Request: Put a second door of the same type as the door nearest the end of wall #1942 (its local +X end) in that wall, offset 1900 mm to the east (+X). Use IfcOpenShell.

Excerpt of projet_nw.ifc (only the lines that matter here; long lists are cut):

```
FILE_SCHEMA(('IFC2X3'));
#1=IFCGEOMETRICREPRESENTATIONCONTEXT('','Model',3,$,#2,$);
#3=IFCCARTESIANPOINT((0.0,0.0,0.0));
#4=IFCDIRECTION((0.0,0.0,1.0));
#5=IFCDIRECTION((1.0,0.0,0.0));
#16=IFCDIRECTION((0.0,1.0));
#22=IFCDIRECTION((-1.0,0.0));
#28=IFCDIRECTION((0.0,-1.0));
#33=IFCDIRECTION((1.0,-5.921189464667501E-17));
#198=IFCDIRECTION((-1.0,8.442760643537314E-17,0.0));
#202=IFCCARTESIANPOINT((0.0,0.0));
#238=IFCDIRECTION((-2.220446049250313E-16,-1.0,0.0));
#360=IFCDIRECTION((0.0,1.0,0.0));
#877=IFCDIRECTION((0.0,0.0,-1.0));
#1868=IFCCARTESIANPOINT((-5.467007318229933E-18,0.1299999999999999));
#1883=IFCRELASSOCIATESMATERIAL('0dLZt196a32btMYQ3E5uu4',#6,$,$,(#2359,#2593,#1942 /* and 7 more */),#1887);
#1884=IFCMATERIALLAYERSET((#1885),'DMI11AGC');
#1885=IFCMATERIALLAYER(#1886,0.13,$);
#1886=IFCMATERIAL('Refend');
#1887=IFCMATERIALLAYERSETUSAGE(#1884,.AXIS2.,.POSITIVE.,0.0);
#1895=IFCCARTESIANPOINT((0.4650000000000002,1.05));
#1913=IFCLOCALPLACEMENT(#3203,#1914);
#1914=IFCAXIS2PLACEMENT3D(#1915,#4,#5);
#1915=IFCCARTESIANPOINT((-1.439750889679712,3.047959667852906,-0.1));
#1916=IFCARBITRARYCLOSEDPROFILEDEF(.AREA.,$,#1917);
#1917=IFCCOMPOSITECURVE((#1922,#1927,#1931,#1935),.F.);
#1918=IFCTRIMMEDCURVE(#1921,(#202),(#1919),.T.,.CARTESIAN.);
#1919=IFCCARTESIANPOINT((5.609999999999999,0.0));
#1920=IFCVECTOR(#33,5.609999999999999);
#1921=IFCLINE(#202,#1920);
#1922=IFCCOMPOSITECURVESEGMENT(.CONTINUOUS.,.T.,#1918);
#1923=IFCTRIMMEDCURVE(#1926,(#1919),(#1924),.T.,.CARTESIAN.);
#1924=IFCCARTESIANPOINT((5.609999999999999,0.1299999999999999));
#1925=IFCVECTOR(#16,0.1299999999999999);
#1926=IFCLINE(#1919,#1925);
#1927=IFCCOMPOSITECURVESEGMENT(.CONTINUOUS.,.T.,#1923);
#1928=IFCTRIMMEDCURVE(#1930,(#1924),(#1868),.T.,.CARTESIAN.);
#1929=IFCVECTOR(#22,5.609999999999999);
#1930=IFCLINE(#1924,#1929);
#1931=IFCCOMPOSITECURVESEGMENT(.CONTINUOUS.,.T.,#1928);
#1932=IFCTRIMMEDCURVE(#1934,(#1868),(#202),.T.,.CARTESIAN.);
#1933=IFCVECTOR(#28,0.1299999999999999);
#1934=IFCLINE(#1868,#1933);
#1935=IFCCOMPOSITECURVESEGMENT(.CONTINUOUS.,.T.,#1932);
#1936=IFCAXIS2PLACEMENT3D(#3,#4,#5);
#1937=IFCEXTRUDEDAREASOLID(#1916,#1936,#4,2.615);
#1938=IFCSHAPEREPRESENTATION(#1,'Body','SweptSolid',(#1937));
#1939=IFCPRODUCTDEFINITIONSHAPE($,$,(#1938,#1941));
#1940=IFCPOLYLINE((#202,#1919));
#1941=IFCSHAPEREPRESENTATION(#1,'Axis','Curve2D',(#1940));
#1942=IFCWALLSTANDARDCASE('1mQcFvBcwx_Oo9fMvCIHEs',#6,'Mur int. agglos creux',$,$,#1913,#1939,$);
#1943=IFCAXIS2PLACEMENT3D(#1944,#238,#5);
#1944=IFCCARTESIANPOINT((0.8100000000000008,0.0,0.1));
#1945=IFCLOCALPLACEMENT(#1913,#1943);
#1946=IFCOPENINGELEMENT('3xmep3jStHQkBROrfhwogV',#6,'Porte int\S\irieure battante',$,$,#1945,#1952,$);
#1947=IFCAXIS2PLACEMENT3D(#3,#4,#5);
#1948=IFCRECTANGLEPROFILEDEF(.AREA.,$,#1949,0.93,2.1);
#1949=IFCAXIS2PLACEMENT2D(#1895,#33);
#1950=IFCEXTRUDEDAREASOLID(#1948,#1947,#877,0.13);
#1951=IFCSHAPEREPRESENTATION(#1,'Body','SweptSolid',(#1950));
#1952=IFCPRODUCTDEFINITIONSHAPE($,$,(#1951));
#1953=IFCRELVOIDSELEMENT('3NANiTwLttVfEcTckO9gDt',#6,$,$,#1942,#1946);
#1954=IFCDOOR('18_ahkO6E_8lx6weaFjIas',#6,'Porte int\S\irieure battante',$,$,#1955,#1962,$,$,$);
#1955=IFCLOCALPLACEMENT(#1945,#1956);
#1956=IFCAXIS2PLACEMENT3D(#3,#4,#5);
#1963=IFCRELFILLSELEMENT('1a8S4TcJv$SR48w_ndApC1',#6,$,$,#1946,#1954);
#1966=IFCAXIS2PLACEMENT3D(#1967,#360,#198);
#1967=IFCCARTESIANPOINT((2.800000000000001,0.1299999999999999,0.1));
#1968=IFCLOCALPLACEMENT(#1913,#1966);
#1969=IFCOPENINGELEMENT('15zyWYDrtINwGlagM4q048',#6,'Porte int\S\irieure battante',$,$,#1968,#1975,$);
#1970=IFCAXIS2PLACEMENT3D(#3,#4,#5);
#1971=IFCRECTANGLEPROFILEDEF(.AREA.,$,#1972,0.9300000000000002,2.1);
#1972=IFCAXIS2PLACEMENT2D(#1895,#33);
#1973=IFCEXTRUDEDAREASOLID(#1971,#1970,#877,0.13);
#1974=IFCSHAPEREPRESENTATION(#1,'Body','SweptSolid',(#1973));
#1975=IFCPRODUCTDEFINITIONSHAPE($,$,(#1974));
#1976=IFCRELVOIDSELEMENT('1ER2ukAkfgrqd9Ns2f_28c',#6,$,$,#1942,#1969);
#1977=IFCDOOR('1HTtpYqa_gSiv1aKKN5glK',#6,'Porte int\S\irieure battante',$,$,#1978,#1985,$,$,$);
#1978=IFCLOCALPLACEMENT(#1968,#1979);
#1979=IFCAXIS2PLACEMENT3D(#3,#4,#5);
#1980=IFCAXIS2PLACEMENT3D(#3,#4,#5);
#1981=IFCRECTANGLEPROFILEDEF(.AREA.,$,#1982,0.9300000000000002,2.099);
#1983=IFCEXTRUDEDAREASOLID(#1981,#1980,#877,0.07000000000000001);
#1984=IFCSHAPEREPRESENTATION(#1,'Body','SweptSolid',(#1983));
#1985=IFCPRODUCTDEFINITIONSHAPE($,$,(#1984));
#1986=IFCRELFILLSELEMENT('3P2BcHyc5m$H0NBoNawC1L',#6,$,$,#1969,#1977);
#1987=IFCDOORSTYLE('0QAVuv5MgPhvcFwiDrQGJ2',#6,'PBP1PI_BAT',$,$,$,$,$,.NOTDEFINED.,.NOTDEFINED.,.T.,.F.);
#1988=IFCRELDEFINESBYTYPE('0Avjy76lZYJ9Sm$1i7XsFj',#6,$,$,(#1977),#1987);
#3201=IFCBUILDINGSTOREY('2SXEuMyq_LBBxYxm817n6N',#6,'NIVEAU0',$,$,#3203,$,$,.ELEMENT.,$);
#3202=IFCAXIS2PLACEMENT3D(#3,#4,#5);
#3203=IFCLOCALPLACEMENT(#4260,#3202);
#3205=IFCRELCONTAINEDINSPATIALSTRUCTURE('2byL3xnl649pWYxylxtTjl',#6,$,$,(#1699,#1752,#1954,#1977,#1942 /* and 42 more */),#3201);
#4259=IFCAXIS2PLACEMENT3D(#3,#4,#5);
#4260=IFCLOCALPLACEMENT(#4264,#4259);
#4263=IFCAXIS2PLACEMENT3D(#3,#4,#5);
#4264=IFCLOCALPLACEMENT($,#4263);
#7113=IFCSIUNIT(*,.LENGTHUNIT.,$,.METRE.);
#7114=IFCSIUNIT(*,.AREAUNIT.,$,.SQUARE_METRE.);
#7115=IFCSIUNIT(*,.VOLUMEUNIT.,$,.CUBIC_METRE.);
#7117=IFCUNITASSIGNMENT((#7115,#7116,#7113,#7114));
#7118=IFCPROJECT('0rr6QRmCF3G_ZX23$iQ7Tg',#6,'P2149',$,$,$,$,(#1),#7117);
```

```python
import ifcopenshell
import ifcopenshell.api.feature
import ifcopenshell.api.geometry
import ifcopenshell.api.root
import ifcopenshell.geom
import ifcopenshell.util.element
import ifcopenshell.util.placement
import ifcopenshell.util.shape
import ifcopenshell.util.unit

model = ifcopenshell.open("projet_nw.ifc")
unit_scale = ifcopenshell.util.unit.calculate_unit_scale(model)
settings = ifcopenshell.geom.settings()


def volume(element):
    """Net volume in cubic metres, openings subtracted."""
    shape = ifcopenshell.geom.create_shape(settings, element)
    return ifcopenshell.util.shape.get_volume(shape.geometry)


door = model.by_guid("1HTtpYqa_gSiv1aKKN5glK")
opening = door.FillsVoids[0].RelatingOpeningElement
wall = opening.VoidsElements[0].RelatingBuildingElement
before = volume(wall)
shift = ifcopenshell.util.placement.get_local_placement(wall.ObjectPlacement)[:3, 0] * 1.9 / unit_scale

# copy_class copies the void relationship, type, container and properties, but no geometry.
new_opening = ifcopenshell.api.root.copy_class(model, product=opening)
new_opening.Representation = ifcopenshell.util.element.copy_deep(
    model, opening.Representation, exclude=["IfcGeometricRepresentationContext", "IfcRepresentationMap"]
)
new_door = ifcopenshell.api.root.copy_class(model, product=door)
new_door.Representation = ifcopenshell.util.element.copy_deep(
    model, door.Representation, exclude=["IfcGeometricRepresentationContext", "IfcRepresentationMap"]
)
fills = ifcopenshell.api.feature.add_filling(model, opening=new_opening, element=new_door)
fills.OwnerHistory = new_door.OwnerHistory  # required in IFC2X3

for old, new in ((opening, new_opening), (door, new_door)):
    matrix = ifcopenshell.util.placement.get_local_placement(old.ObjectPlacement)
    matrix[:3, 3] += shift
    ifcopenshell.api.geometry.edit_object_placement(model, product=new, matrix=matrix, is_si=False)

after = volume(wall)

print(f"wall volume {before:.3f} -> {after:.3f} m3")

model.write("projet_nw-out.ifc")
```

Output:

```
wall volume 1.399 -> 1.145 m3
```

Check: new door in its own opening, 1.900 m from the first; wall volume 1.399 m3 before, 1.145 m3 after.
